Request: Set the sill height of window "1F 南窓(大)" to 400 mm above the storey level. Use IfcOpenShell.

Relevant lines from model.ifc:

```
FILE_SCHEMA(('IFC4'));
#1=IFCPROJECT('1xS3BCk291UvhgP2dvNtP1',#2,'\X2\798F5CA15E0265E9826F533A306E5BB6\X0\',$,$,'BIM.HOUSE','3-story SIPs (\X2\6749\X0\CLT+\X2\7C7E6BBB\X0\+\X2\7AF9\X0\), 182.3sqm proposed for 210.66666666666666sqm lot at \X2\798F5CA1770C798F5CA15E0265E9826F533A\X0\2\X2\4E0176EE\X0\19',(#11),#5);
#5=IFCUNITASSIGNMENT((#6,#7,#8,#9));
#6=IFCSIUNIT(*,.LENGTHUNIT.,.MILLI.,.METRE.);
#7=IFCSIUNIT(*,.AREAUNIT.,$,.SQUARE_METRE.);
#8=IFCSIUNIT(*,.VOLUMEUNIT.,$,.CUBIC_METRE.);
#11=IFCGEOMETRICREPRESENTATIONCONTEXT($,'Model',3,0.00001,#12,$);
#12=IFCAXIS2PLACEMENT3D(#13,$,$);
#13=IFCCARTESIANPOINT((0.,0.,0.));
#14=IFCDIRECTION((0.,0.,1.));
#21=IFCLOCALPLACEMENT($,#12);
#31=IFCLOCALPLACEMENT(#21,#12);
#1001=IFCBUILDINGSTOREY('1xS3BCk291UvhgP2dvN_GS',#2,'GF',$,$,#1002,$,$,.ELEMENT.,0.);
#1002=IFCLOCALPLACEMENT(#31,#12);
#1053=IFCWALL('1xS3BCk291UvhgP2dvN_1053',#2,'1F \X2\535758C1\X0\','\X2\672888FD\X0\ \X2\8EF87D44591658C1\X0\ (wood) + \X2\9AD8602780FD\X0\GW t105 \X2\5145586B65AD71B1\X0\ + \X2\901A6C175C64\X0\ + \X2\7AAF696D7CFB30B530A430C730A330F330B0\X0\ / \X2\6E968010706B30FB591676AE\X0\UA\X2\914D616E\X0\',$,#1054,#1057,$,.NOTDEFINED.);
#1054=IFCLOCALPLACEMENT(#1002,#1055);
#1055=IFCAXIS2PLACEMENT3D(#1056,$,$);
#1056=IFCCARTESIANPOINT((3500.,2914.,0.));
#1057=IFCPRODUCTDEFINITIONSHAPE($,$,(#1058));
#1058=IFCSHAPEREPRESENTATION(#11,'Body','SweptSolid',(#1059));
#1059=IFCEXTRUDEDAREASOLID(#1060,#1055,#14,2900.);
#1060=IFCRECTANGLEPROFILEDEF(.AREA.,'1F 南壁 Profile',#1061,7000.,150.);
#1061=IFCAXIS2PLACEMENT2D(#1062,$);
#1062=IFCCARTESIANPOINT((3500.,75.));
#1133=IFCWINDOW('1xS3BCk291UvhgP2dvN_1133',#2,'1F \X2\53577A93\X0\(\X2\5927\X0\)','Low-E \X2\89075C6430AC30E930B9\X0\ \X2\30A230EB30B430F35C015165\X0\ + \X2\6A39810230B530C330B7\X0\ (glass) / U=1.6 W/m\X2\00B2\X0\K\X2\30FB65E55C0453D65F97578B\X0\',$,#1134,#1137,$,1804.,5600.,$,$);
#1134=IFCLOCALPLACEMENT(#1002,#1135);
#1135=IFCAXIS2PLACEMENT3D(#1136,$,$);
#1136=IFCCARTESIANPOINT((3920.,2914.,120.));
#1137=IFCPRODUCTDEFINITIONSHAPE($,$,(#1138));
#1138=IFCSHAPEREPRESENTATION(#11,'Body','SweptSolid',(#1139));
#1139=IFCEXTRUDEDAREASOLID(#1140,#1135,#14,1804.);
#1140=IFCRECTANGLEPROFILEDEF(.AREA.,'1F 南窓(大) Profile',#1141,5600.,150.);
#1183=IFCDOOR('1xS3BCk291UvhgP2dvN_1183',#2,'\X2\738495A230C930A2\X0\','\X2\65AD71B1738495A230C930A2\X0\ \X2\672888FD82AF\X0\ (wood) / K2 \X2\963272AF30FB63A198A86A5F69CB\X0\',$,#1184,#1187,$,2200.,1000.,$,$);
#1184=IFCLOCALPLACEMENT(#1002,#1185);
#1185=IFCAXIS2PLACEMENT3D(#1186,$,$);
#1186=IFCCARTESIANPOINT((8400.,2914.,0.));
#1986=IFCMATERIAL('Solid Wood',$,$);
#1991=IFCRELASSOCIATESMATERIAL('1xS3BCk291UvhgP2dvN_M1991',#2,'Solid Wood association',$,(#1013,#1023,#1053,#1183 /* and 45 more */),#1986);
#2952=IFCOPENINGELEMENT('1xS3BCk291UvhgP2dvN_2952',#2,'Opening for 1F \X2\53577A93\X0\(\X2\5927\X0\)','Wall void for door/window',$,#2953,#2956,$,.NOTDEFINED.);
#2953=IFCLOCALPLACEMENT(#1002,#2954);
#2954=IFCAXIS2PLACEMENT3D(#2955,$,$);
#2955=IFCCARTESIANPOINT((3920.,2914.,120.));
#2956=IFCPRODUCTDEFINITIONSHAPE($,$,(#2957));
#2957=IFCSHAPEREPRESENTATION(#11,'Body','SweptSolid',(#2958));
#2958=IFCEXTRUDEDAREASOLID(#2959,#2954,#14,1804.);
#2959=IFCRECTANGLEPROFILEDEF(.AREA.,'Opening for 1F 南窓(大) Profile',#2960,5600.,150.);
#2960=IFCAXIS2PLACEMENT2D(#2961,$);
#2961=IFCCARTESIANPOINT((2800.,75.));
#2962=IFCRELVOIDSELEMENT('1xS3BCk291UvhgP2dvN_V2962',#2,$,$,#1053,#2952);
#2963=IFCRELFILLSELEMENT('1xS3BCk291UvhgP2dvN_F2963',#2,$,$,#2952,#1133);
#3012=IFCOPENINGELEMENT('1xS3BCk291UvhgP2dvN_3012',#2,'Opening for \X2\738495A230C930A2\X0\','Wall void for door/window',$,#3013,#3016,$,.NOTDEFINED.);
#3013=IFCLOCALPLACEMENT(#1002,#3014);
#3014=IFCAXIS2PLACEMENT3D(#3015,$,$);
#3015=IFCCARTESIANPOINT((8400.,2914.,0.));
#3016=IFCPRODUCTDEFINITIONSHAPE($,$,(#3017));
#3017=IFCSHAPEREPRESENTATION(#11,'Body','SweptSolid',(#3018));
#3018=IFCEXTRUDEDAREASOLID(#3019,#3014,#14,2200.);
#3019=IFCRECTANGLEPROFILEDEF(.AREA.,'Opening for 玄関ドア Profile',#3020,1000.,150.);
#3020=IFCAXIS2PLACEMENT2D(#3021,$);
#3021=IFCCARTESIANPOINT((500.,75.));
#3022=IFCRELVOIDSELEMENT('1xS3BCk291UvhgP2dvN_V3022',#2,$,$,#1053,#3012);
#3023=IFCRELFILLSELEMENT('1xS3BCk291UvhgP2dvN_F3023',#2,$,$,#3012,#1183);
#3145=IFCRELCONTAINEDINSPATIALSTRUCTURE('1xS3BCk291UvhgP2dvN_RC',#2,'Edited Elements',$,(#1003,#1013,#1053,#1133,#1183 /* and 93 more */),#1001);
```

```python
import numpy as np
import ifcopenshell
import ifcopenshell.api.geometry
import ifcopenshell.geom
import ifcopenshell.util.element
import ifcopenshell.util.placement
import ifcopenshell.util.shape
import ifcopenshell.util.unit

model = ifcopenshell.open("model.ifc")
unit_scale = ifcopenshell.util.unit.calculate_unit_scale(model)

window = model.by_guid("1xS3BCk291UvhgP2dvN_1133")
opening = window.FillsVoids[0].RelatingOpeningElement
storey = ifcopenshell.util.element.get_container(window, ifc_class="IfcBuildingStorey")
level = ifcopenshell.util.placement.get_local_placement(storey.ObjectPlacement)[2, 3]

# The opening's origin need not be at the sill, so measure its lowest point.
shape = ifcopenshell.geom.create_shape(ifcopenshell.geom.settings(), opening)
bottom = ifcopenshell.util.shape.get_shape_bottom_elevation(shape, shape.geometry) / unit_scale
dz = level + 0.4 / unit_scale - bottom

shift = np.array([0.0, 0.0, dz])
# The window is not placed relative to its opening, so move both.
for product in (opening, window):
    matrix = ifcopenshell.util.placement.get_local_placement(product.ObjectPlacement)
    matrix[:3, 3] += shift
    ifcopenshell.api.geometry.edit_object_placement(model, product=product, matrix=matrix, is_si=False)

print(f"moved by {dz * unit_scale:+.3f} m")

model.write("model_edited.ifc")
```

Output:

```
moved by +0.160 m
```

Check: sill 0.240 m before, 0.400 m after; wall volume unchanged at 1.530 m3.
